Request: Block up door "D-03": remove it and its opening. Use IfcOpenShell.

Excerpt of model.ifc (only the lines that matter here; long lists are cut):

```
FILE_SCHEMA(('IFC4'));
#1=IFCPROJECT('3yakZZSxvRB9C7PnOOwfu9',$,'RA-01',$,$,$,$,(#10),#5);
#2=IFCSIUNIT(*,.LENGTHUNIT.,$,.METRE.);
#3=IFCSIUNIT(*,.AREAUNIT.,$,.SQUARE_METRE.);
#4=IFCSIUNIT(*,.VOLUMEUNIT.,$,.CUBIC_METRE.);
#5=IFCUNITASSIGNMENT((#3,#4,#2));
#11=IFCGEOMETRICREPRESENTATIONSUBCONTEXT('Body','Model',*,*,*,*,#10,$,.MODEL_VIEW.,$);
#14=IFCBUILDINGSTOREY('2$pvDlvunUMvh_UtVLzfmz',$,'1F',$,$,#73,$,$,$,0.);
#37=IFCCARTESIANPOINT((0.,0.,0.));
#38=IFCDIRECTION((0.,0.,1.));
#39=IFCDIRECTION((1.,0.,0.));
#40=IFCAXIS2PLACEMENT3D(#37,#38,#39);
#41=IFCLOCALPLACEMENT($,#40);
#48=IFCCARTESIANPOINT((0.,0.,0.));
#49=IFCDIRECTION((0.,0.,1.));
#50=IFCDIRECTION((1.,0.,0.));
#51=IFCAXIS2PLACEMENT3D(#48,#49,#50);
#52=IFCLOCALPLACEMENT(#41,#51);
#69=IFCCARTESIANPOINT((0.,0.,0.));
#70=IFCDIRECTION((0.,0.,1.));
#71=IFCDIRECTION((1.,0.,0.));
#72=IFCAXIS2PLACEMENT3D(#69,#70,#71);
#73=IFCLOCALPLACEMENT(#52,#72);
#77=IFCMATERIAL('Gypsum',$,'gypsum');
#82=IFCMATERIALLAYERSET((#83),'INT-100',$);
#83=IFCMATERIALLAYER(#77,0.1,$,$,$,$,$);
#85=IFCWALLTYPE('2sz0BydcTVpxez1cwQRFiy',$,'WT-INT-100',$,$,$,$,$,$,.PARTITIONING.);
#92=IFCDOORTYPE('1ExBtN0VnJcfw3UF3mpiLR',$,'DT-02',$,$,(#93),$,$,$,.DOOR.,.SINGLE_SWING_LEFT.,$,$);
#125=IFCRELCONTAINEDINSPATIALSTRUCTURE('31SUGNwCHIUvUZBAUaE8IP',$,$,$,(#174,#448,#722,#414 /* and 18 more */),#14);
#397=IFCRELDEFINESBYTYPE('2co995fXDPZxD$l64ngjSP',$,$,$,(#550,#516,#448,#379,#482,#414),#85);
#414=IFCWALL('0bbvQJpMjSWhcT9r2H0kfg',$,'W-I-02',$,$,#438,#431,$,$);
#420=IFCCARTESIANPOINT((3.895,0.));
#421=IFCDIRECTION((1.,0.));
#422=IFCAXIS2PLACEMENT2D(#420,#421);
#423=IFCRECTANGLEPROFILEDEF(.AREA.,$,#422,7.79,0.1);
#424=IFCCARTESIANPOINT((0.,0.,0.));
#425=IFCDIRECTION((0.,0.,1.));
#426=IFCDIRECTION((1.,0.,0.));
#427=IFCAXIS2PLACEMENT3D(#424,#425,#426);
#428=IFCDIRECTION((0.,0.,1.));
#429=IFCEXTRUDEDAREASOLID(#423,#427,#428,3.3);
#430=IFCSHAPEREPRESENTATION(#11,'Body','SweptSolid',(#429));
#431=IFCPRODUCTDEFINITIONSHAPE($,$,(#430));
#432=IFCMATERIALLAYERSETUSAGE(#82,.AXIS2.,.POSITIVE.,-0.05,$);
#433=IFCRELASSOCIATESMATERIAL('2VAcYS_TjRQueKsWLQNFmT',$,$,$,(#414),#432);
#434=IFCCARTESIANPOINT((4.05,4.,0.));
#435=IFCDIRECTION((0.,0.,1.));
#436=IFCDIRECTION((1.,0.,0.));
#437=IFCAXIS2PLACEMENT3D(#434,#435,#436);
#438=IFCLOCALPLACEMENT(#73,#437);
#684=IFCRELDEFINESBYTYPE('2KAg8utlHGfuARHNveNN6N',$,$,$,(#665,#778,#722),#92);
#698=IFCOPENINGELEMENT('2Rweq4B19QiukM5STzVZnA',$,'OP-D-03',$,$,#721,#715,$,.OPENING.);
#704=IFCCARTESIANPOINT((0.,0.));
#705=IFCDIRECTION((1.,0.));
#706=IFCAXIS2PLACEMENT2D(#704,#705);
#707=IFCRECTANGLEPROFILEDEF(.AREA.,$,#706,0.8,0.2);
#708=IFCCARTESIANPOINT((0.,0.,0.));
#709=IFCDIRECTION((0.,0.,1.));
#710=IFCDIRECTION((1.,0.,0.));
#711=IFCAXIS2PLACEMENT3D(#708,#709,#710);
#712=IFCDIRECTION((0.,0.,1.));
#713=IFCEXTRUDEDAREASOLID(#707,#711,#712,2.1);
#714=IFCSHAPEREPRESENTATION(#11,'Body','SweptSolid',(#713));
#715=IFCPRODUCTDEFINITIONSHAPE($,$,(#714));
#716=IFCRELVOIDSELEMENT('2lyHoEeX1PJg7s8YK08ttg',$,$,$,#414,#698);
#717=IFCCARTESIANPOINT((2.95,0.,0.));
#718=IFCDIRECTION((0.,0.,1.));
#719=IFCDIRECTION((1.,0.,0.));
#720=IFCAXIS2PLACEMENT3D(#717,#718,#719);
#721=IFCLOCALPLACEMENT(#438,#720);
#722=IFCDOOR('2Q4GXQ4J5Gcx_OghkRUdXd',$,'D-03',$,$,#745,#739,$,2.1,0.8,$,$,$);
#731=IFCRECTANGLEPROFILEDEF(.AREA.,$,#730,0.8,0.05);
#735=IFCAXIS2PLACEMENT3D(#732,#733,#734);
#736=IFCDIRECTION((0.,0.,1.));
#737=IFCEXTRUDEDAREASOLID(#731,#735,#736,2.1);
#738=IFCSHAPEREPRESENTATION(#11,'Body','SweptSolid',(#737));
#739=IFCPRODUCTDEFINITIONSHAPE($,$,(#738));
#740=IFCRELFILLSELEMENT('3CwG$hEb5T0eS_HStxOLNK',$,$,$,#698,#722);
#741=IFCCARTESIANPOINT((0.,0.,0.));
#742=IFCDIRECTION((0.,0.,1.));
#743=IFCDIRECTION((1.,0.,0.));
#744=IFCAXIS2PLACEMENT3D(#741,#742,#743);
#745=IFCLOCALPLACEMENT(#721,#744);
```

```python
import ifcopenshell
import ifcopenshell.api.feature
import ifcopenshell.api.root
import ifcopenshell.geom
import ifcopenshell.util.shape

model = ifcopenshell.open("model.ifc")
settings = ifcopenshell.geom.settings()


def volume(element):
    """Net volume in cubic metres, openings subtracted."""
    shape = ifcopenshell.geom.create_shape(settings, element)
    return ifcopenshell.util.shape.get_volume(shape.geometry)


door = model.by_id(722)
opening = door.FillsVoids[0].RelatingOpeningElement
wall = opening.VoidsElements[0].RelatingBuildingElement
before = volume(wall)

ifcopenshell.api.root.remove_product(model, product=door)
ifcopenshell.api.feature.remove_feature(model, feature=opening)

after = volume(wall)

print(f"wall volume {before:.3f} -> {after:.3f} m3")

model.write("model_updated.ifc")
```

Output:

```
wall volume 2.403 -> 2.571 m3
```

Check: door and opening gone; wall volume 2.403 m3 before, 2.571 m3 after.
